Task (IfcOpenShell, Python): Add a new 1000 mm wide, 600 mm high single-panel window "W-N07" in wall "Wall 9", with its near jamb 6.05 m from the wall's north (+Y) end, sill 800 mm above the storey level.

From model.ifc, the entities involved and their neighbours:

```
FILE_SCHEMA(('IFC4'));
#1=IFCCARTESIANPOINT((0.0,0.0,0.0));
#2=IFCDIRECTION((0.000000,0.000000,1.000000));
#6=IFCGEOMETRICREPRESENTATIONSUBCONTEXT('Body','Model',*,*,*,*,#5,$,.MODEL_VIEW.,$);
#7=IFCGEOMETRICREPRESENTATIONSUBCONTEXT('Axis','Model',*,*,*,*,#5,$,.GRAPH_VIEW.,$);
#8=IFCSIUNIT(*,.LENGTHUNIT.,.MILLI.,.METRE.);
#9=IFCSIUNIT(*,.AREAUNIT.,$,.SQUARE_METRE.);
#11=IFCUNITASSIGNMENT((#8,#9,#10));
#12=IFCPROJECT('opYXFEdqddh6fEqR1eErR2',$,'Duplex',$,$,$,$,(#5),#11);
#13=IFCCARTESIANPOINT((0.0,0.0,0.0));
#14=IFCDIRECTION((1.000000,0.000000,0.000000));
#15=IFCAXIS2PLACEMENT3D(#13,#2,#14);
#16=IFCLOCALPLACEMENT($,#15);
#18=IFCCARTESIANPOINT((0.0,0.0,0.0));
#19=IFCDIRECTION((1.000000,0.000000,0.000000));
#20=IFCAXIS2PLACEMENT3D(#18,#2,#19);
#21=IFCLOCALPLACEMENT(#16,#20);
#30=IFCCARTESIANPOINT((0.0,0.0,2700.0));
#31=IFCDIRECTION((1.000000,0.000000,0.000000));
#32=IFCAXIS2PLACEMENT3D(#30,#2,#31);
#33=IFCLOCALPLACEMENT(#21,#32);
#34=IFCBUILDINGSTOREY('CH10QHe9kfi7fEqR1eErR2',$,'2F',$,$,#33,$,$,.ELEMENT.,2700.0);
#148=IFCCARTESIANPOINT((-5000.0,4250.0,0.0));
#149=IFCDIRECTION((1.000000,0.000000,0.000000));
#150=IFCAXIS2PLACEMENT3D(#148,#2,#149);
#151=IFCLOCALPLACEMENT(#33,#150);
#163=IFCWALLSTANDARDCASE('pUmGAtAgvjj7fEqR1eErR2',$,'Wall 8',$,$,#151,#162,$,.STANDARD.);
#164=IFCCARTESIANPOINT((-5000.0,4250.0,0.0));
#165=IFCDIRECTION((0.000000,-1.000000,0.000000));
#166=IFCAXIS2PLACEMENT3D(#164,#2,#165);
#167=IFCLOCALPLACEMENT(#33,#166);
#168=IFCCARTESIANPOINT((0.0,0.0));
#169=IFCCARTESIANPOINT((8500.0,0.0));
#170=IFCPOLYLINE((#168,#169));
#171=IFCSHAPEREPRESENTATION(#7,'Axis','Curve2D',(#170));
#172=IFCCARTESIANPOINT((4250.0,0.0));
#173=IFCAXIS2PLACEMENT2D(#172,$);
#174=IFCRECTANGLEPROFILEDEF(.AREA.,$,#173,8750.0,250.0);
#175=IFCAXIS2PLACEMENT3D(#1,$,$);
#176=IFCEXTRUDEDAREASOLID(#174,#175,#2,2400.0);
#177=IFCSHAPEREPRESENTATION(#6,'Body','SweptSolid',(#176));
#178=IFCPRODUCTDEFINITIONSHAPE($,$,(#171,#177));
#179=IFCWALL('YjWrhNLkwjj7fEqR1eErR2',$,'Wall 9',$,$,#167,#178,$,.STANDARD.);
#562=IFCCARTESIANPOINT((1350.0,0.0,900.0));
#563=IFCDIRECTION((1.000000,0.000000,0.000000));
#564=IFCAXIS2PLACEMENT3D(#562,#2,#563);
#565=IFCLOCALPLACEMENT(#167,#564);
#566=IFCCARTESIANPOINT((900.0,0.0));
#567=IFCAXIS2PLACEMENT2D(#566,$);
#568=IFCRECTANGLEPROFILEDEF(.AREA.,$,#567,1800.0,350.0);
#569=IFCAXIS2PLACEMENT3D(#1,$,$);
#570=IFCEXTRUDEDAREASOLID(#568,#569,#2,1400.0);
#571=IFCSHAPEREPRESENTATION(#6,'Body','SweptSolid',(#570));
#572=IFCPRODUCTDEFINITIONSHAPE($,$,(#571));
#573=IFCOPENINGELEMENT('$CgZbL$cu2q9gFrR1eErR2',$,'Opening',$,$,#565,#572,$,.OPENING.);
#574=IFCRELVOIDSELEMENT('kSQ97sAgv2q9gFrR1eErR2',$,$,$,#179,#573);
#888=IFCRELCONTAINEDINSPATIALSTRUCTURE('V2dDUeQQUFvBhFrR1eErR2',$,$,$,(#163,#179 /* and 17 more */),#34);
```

```python
import numpy as np
import ifcopenshell
import ifcopenshell.api.feature
import ifcopenshell.api.geometry
import ifcopenshell.api.root
import ifcopenshell.api.spatial
import ifcopenshell.geom
import ifcopenshell.util.element
import ifcopenshell.util.placement
import ifcopenshell.util.representation
import ifcopenshell.util.shape
import ifcopenshell.util.unit

model = ifcopenshell.open("model.ifc")
unit_scale = ifcopenshell.util.unit.calculate_unit_scale(model)
settings = ifcopenshell.geom.settings()


def volume(element):
    """Net volume in cubic metres, openings subtracted."""
    shape = ifcopenshell.geom.create_shape(settings, element)
    return ifcopenshell.util.shape.get_volume(shape.geometry)


wall = model.by_id(179)
storey = ifcopenshell.util.element.get_container(wall, ifc_class="IfcBuildingStorey")
context = ifcopenshell.util.representation.get_context(model, "Model", "Body", "MODEL_VIEW")
before = volume(wall)

width, height, from_end, sill = 1, 0.6, 6.05, 0.8  # metres

# The wall runs along its own X axis, and the end named is its -X end.
wall_shape = ifcopenshell.geom.create_shape(settings, wall)
x, y, z = ifcopenshell.util.shape.get_vertices(wall_shape.geometry).T
start = x.min() + from_end
face, thickness = float(y.min()), float(y.max() - y.min())
wall_matrix = ifcopenshell.util.placement.get_local_placement(wall.ObjectPlacement)
level = ifcopenshell.util.placement.get_local_placement(storey.ObjectPlacement)[2, 3]


def in_wall(x, y):
    """Placement at x, y metres in the wall's axes, at sill height."""
    matrix = wall_matrix.copy()
    matrix[:, 3] = wall_matrix @ np.array([x / unit_scale, y / unit_scale, 0.0, 1.0])
    matrix[2, 3] = level + sill / unit_scale
    return matrix


# Opening: a box that overshoots both wall faces by 50 mm.
opening = ifcopenshell.api.root.create_entity(model, ifc_class="IfcOpeningElement", predefined_type="OPENING")
box = ifcopenshell.api.geometry.add_wall_representation(
    model, context=context, length=width, height=height, thickness=thickness + 0.1
)
ifcopenshell.api.geometry.assign_representation(model, product=opening, representation=box)
ifcopenshell.api.geometry.edit_object_placement(model, product=opening, matrix=in_wall(start, face - 0.05), is_si=False)
ifcopenshell.api.feature.add_feature(model, feature=opening, element=wall)

window = ifcopenshell.api.root.create_entity(model, ifc_class="IfcWindow", name="W-N07", predefined_type="WINDOW")
window.OverallWidth, window.OverallHeight = width / unit_scale, height / unit_scale
window.PartitioningType = "SINGLE_PANEL"
body = ifcopenshell.api.geometry.add_window_representation(
    model,
    context=context,
    overall_width=window.OverallWidth,
    overall_height=window.OverallHeight,
    partition_type="SINGLE_PANEL",
)
ifcopenshell.api.geometry.assign_representation(model, product=window, representation=body)
ifcopenshell.api.spatial.assign_container(model, products=[window], relating_structure=storey)
ifcopenshell.api.feature.add_filling(model, opening=opening, element=window)

# Centre the window in the wall's thickness.
ifcopenshell.api.geometry.edit_object_placement(model, product=window, matrix=in_wall(start, face), is_si=False)
window_shape = ifcopenshell.geom.create_shape(settings, window)
depth = ifcopenshell.util.shape.get_vertices(window_shape.geometry)[:, 1]
offset = face + thickness / 2 - (depth.min() + depth.max()) / 2
ifcopenshell.api.geometry.edit_object_placement(model, product=window, matrix=in_wall(start, offset), is_si=False)

after = volume(wall)

print(f"wall volume {before:.3f} -> {after:.3f} m3")

model.write("model_v2.ifc")
```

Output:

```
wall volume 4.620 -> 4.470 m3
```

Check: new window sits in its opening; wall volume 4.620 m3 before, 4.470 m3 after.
